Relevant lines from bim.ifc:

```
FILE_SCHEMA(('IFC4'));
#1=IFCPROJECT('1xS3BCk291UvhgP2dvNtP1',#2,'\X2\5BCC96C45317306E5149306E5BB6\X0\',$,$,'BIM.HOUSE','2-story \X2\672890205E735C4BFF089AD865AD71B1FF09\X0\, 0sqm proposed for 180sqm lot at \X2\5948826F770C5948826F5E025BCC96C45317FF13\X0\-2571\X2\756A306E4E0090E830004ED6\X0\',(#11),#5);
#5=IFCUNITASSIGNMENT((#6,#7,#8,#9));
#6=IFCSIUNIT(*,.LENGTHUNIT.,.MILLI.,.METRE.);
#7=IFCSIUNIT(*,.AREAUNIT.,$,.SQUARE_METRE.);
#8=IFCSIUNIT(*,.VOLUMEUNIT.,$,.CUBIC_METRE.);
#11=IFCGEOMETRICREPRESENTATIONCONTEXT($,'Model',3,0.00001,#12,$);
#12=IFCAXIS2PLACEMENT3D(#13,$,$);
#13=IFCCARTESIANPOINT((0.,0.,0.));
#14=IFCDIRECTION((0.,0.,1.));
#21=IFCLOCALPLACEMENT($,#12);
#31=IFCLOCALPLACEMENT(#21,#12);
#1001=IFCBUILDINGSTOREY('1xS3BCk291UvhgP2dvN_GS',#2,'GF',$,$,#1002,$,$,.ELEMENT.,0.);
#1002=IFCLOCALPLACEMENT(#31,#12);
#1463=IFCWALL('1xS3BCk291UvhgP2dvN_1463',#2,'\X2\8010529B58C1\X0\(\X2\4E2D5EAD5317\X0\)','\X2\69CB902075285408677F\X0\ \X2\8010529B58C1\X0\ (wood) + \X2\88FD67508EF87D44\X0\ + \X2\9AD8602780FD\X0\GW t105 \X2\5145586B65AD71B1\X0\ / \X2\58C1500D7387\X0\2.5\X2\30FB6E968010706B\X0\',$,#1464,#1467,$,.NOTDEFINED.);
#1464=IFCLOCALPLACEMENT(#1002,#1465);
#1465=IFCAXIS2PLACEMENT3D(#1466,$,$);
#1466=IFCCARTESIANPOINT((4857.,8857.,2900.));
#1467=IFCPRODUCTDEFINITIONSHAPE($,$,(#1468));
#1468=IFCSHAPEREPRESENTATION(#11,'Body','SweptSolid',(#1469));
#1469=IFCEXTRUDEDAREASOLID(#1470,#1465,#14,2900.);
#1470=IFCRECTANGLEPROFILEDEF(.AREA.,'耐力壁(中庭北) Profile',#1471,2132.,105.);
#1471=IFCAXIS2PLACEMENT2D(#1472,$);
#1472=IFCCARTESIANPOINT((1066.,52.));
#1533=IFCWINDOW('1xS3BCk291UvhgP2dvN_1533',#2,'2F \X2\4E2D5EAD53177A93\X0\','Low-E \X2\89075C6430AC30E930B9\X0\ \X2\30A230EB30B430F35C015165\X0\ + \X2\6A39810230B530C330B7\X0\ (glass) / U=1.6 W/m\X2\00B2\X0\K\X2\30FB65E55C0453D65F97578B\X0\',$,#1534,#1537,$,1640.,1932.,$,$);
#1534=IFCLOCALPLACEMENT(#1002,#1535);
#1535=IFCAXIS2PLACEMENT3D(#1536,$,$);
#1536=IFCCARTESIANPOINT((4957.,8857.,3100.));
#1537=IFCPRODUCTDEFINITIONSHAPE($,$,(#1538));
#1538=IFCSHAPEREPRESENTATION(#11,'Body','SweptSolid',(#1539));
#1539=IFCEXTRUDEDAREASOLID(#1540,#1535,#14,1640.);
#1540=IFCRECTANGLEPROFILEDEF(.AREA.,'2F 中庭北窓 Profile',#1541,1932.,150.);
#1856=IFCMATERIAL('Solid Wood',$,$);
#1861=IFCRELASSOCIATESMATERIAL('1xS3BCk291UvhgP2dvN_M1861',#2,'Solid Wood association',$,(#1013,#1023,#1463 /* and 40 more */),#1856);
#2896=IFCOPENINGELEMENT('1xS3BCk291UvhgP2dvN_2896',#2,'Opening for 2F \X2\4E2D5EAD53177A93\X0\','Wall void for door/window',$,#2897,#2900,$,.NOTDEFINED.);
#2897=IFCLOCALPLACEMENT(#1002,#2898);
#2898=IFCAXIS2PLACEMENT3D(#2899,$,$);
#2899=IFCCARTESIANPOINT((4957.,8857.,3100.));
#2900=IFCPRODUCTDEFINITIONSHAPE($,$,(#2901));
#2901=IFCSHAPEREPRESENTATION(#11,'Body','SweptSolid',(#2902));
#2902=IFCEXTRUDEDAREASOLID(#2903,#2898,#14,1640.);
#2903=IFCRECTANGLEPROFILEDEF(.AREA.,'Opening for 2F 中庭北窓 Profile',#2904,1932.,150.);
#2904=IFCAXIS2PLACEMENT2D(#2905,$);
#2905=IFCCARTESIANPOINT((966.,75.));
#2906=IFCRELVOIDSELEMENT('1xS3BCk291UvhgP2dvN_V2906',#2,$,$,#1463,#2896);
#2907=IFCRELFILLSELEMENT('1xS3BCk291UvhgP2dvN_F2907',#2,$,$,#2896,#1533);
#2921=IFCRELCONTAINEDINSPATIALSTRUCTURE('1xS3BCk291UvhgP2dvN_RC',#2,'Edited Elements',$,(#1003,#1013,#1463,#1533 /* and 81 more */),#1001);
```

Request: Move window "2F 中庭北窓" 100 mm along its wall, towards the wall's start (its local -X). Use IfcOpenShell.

```python
import ifcopenshell
import ifcopenshell.api.geometry
import ifcopenshell.util.placement

model = ifcopenshell.open("bim.ifc")

window = model.by_id(1533)
opening = window.FillsVoids[0].RelatingOpeningElement
wall = opening.VoidsElements[0].RelatingBuildingElement

wall_matrix = ifcopenshell.util.placement.get_local_placement(wall.ObjectPlacement)
shift = wall_matrix[:3, 0] * -100.0
before = ifcopenshell.util.placement.get_local_placement(window.ObjectPlacement)[:3, 3].copy()

# The window is not placed relative to its opening, so move both.
for product in (opening, window):
    matrix = ifcopenshell.util.placement.get_local_placement(product.ObjectPlacement)
    matrix[:3, 3] += shift
    ifcopenshell.api.geometry.edit_object_placement(model, product=product, matrix=matrix, is_si=False)

after = ifcopenshell.util.placement.get_local_placement(window.ObjectPlacement)[:3, 3]
print("window moved by", (after - before).round(3) + 0.0)

model.write("bim_edited.ifc")
```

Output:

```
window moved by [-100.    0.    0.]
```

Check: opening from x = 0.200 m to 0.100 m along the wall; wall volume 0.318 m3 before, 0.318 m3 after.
